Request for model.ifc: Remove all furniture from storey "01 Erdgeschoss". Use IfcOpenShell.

First a look at what the model holds.

```python
import ifcopenshell
import ifcopenshell.util.element

model = ifcopenshell.open("model.ifc")
print(model.schema)
storey = next(s for s in model.by_type("IfcBuildingStorey") if s.Name == "01 Erdgeschoss")
furniture = [e for e in ifcopenshell.util.element.get_decomposition(storey) if e.is_a("IfcFurnishingElement")]
seen = {}
for e in furniture:
    element_type = ifcopenshell.util.element.get_type(e)
    name = element_type.Name if element_type not in (None, e) else None
    seen[name] = seen.get(name, 0) + 1
for name, count in sorted(seen.items(), key=str):
    print(count, "x", name)
```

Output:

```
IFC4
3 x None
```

```python
import ifcopenshell
import ifcopenshell.api.root
import ifcopenshell.util.element

model = ifcopenshell.open("model.ifc")

storey = next(s for s in model.by_type("IfcBuildingStorey") if s.Name == "01 Erdgeschoss")
furniture = [e for e in ifcopenshell.util.element.get_decomposition(storey) if e.is_a("IfcFurnishingElement")]

for e in furniture:
    ifcopenshell.api.root.remove_product(model, product=e)
print(len(furniture), "removed")

model.write("model_v2.ifc")
```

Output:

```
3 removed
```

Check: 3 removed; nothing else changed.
